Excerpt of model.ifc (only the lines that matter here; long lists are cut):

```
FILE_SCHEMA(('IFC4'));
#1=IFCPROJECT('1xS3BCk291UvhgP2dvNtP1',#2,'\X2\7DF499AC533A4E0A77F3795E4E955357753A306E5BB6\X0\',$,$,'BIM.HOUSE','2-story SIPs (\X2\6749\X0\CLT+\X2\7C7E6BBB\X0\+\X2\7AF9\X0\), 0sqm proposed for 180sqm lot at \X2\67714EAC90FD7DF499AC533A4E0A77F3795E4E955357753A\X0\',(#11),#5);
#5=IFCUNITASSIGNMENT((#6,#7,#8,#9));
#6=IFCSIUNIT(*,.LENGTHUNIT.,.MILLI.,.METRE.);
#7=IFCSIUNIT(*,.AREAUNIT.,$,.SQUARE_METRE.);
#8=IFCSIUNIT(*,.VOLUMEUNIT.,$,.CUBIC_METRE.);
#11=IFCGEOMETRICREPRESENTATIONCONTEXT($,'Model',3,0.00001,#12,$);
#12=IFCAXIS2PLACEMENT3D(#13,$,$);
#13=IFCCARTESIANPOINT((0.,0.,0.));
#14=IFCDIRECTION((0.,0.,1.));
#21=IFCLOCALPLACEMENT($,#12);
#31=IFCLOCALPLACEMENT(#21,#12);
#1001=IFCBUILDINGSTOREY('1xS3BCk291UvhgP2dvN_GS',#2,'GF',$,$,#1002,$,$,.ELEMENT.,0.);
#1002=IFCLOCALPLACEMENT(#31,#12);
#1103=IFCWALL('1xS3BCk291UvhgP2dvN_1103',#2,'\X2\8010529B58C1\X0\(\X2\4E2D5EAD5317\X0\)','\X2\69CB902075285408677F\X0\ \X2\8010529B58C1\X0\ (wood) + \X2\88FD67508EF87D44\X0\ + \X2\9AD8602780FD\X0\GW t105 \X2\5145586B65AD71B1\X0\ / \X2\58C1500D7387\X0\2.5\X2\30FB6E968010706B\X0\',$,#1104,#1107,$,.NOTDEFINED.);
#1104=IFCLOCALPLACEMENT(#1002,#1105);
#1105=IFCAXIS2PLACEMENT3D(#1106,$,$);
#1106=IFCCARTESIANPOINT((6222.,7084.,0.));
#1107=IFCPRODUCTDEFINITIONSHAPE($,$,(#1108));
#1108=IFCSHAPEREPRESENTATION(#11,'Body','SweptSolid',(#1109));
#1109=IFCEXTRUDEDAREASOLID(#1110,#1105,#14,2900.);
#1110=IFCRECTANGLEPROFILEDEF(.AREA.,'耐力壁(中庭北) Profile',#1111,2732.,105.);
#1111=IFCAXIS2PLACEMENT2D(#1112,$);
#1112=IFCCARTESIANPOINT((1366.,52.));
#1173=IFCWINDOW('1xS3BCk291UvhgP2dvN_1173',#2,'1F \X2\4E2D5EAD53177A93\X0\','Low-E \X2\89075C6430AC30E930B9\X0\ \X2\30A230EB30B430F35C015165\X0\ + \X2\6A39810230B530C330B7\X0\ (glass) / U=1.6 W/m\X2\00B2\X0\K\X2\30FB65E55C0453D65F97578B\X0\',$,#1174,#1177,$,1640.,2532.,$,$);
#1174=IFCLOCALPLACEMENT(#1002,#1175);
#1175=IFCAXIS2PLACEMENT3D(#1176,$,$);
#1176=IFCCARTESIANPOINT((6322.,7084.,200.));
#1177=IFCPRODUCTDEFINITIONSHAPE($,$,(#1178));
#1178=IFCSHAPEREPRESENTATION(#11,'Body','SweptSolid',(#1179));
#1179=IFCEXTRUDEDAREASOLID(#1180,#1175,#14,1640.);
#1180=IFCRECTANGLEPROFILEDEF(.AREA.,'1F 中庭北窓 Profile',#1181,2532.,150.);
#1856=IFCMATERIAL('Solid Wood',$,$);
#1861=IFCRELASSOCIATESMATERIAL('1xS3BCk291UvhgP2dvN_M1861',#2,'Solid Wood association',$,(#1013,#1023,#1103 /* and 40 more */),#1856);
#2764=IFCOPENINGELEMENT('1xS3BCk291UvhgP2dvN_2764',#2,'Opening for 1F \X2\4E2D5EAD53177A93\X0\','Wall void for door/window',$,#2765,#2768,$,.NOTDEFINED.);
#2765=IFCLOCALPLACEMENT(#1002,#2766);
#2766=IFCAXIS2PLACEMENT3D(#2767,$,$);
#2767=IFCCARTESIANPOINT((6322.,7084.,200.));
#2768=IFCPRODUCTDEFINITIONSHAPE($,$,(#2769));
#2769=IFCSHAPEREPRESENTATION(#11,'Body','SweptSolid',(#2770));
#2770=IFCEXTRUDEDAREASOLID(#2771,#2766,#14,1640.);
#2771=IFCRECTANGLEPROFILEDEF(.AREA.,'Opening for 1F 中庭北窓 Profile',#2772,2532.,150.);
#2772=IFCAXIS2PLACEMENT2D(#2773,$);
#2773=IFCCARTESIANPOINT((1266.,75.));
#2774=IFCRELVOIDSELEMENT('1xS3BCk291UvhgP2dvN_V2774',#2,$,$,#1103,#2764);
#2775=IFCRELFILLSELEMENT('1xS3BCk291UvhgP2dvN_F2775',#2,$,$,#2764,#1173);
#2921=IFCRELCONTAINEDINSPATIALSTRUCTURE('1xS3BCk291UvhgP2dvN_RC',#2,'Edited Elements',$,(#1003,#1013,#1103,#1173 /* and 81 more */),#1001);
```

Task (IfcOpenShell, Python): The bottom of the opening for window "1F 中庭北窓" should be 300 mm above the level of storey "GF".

```python
import numpy as np
import ifcopenshell
import ifcopenshell.api.geometry
import ifcopenshell.geom
import ifcopenshell.util.element
import ifcopenshell.util.placement
import ifcopenshell.util.shape
import ifcopenshell.util.unit

model = ifcopenshell.open("model.ifc")
unit_scale = ifcopenshell.util.unit.calculate_unit_scale(model)

window = model.by_id(1173)
opening = window.FillsVoids[0].RelatingOpeningElement
storey = ifcopenshell.util.element.get_container(window, ifc_class="IfcBuildingStorey")
level = ifcopenshell.util.placement.get_local_placement(storey.ObjectPlacement)[2, 3]

# The opening's origin need not be at the sill, so measure its lowest point.
shape = ifcopenshell.geom.create_shape(ifcopenshell.geom.settings(), opening)
bottom = ifcopenshell.util.shape.get_shape_bottom_elevation(shape, shape.geometry) / unit_scale
dz = level + 0.3 / unit_scale - bottom

shift = np.array([0.0, 0.0, dz])
# The window is not placed relative to its opening, so move both.
for product in (opening, window):
    matrix = ifcopenshell.util.placement.get_local_placement(product.ObjectPlacement)
    matrix[:3, 3] += shift
    ifcopenshell.api.geometry.edit_object_placement(model, product=product, matrix=matrix, is_si=False)

print(f"moved by {dz * unit_scale:+.3f} m")

model.write("model_rev.ifc")
```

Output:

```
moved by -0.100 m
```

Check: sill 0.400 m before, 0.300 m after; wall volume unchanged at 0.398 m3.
